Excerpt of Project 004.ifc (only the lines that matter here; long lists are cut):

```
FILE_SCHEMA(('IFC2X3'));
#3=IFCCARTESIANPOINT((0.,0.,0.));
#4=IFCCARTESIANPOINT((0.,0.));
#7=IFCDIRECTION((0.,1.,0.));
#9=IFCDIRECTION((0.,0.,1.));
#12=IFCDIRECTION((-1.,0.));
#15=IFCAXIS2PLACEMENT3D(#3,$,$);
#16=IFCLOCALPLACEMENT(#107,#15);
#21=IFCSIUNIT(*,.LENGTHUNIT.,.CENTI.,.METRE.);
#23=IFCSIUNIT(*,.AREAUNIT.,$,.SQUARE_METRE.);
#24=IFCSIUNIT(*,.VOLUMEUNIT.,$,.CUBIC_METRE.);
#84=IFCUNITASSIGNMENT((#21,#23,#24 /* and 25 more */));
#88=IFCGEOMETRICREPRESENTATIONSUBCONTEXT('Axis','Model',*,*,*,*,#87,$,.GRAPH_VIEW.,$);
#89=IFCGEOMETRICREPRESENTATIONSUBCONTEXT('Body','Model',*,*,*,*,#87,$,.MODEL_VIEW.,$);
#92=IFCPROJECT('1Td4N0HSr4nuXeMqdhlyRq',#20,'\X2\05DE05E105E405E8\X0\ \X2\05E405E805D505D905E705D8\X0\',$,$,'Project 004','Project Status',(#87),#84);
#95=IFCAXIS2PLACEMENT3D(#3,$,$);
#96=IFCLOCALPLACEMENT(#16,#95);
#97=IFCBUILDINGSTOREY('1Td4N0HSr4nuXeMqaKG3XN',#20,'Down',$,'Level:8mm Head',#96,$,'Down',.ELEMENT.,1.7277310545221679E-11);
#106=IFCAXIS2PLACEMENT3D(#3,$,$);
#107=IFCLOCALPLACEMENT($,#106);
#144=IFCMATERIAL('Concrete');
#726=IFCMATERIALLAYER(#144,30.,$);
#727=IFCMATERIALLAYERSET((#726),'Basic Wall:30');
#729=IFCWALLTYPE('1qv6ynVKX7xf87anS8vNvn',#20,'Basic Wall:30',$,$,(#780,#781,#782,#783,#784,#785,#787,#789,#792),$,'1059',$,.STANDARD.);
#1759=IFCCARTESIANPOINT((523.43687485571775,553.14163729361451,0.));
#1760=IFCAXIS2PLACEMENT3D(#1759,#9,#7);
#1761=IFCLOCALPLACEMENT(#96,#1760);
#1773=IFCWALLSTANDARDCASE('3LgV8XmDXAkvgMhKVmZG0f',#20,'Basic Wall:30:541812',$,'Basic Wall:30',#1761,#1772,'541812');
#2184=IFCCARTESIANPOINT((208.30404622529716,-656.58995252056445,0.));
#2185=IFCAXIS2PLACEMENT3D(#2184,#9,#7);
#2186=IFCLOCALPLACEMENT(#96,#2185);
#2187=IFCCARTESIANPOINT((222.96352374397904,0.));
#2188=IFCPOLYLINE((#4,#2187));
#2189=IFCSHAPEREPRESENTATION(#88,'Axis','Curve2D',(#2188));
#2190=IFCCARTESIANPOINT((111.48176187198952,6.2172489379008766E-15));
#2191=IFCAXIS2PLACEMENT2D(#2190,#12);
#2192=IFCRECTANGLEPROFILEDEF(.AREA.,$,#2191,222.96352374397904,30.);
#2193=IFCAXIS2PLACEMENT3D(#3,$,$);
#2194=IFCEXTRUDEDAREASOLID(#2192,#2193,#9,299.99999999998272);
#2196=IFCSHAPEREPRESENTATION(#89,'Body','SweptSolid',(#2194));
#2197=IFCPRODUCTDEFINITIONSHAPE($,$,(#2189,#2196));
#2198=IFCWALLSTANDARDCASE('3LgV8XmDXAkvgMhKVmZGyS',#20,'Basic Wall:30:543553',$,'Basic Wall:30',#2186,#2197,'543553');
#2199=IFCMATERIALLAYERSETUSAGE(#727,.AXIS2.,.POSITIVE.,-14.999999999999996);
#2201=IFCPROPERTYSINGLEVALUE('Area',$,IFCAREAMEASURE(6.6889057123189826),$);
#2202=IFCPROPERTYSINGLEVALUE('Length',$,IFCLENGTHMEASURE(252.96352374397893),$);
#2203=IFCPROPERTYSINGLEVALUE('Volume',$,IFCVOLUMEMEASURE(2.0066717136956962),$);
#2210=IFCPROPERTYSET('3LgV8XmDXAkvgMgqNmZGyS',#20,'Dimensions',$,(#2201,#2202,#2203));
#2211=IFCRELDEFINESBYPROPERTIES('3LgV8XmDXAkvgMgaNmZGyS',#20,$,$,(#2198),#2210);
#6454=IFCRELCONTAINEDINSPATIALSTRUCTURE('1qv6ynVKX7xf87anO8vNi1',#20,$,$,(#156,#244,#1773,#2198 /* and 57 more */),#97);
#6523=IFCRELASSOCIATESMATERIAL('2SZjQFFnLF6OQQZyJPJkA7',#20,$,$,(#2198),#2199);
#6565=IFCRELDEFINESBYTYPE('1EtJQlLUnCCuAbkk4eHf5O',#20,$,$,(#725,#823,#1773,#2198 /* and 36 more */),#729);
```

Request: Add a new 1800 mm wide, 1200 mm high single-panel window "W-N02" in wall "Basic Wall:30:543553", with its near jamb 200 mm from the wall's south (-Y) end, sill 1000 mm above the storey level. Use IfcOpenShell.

```python
import numpy as np
import ifcopenshell
import ifcopenshell.api.feature
import ifcopenshell.api.geometry
import ifcopenshell.api.pset
import ifcopenshell.api.root
import ifcopenshell.api.spatial
import ifcopenshell.api.type
import ifcopenshell.geom
import ifcopenshell.util.element
import ifcopenshell.util.placement
import ifcopenshell.util.representation
import ifcopenshell.util.shape
import ifcopenshell.util.unit

model = ifcopenshell.open("Project 004.ifc")
unit_scale = ifcopenshell.util.unit.calculate_unit_scale(model)
area_scale = ifcopenshell.util.unit.calculate_unit_scale(model, "AREAUNIT")
volume_scale = ifcopenshell.util.unit.calculate_unit_scale(model, "VOLUMEUNIT")
settings = ifcopenshell.geom.settings()


def volume(element):
    """Net volume in cubic metres, openings subtracted."""
    shape = ifcopenshell.geom.create_shape(settings, element)
    return ifcopenshell.util.shape.get_volume(shape.geometry)


wall = model.by_guid("3LgV8XmDXAkvgMhKVmZGyS")
storey = ifcopenshell.util.element.get_container(wall, ifc_class="IfcBuildingStorey")
context = ifcopenshell.util.representation.get_context(model, "Model", "Body", "MODEL_VIEW")
before = volume(wall)

width, height, from_end, sill = 1.8, 1.2, 0.2, 1  # metres

# The wall runs along its own X axis, and the end named is its -X end.
wall_shape = ifcopenshell.geom.create_shape(settings, wall)
x, y, z = ifcopenshell.util.shape.get_vertices(wall_shape.geometry).T
start = x.min() + from_end
face, thickness = float(y.min()), float(y.max() - y.min())
wall_matrix = ifcopenshell.util.placement.get_local_placement(wall.ObjectPlacement)
level = ifcopenshell.util.placement.get_local_placement(storey.ObjectPlacement)[2, 3]


def in_wall(x, y):
    """Placement at x, y metres in the wall's axes, at sill height."""
    matrix = wall_matrix.copy()
    matrix[:, 3] = wall_matrix @ np.array([x / unit_scale, y / unit_scale, 0.0, 1.0])
    matrix[2, 3] = level + sill / unit_scale
    return matrix


# Opening: a box that overshoots both wall faces by 50 mm.
opening = ifcopenshell.api.root.create_entity(model, ifc_class="IfcOpeningElement")
box = ifcopenshell.api.geometry.add_wall_representation(
    model, context=context, length=width, height=height, thickness=thickness + 0.1
)
ifcopenshell.api.geometry.assign_representation(model, product=opening, representation=box)
ifcopenshell.api.geometry.edit_object_placement(model, product=opening, matrix=in_wall(start, face - 0.05), is_si=False)
ifcopenshell.api.feature.add_feature(model, feature=opening, element=wall)

window = ifcopenshell.api.root.create_entity(model, ifc_class="IfcWindow", name="W-N02")
window.OverallWidth, window.OverallHeight = width / unit_scale, height / unit_scale
body = ifcopenshell.api.geometry.add_window_representation(
    model,
    context=context,
    overall_width=window.OverallWidth,
    overall_height=window.OverallHeight,
    partition_type="SINGLE_PANEL",
)
ifcopenshell.api.geometry.assign_representation(model, product=window, representation=body)
ifcopenshell.api.spatial.assign_container(model, products=[window], relating_structure=storey)
fills = ifcopenshell.api.feature.add_filling(model, opening=opening, element=window)
fills.OwnerHistory = window.OwnerHistory  # required in IFC2X3

# IFC2X3 keeps the operation on the window style.
style = ifcopenshell.api.root.create_entity(model, ifc_class="IfcWindowStyle", name="W-N02")
style.OperationType, style.ConstructionType = "SINGLE_PANEL", "NOTDEFINED"
style.ParameterTakesPrecedence = style.Sizeable = False
ifcopenshell.api.type.assign_type(model, related_objects=[window], relating_type=style)

# Centre the window in the wall's thickness.
ifcopenshell.api.geometry.edit_object_placement(model, product=window, matrix=in_wall(start, face), is_si=False)
window_shape = ifcopenshell.geom.create_shape(settings, window)
depth = ifcopenshell.util.shape.get_vertices(window_shape.geometry)[:, 1]
offset = face + thickness / 2 - (depth.min() + depth.max()) / 2
ifcopenshell.api.geometry.edit_object_placement(model, product=window, matrix=in_wall(start, offset), is_si=False)

after = volume(wall)

# Update the wall's stored quantities.
pset = model.by_id(ifcopenshell.util.element.get_pset(wall, "Dimensions", should_inherit=False)["id"])
ifcopenshell.api.pset.edit_pset(model, pset=pset, properties={
    "Area": model.create_entity("IfcAreaMeasure", after / thickness / area_scale),
    "Volume": model.create_entity("IfcVolumeMeasure", after / volume_scale),
})

print(f"wall volume {before:.3f} -> {after:.3f} m3")

model.write("Project 004_rev.ifc")
```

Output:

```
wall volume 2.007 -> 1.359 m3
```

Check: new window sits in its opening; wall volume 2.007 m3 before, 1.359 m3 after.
